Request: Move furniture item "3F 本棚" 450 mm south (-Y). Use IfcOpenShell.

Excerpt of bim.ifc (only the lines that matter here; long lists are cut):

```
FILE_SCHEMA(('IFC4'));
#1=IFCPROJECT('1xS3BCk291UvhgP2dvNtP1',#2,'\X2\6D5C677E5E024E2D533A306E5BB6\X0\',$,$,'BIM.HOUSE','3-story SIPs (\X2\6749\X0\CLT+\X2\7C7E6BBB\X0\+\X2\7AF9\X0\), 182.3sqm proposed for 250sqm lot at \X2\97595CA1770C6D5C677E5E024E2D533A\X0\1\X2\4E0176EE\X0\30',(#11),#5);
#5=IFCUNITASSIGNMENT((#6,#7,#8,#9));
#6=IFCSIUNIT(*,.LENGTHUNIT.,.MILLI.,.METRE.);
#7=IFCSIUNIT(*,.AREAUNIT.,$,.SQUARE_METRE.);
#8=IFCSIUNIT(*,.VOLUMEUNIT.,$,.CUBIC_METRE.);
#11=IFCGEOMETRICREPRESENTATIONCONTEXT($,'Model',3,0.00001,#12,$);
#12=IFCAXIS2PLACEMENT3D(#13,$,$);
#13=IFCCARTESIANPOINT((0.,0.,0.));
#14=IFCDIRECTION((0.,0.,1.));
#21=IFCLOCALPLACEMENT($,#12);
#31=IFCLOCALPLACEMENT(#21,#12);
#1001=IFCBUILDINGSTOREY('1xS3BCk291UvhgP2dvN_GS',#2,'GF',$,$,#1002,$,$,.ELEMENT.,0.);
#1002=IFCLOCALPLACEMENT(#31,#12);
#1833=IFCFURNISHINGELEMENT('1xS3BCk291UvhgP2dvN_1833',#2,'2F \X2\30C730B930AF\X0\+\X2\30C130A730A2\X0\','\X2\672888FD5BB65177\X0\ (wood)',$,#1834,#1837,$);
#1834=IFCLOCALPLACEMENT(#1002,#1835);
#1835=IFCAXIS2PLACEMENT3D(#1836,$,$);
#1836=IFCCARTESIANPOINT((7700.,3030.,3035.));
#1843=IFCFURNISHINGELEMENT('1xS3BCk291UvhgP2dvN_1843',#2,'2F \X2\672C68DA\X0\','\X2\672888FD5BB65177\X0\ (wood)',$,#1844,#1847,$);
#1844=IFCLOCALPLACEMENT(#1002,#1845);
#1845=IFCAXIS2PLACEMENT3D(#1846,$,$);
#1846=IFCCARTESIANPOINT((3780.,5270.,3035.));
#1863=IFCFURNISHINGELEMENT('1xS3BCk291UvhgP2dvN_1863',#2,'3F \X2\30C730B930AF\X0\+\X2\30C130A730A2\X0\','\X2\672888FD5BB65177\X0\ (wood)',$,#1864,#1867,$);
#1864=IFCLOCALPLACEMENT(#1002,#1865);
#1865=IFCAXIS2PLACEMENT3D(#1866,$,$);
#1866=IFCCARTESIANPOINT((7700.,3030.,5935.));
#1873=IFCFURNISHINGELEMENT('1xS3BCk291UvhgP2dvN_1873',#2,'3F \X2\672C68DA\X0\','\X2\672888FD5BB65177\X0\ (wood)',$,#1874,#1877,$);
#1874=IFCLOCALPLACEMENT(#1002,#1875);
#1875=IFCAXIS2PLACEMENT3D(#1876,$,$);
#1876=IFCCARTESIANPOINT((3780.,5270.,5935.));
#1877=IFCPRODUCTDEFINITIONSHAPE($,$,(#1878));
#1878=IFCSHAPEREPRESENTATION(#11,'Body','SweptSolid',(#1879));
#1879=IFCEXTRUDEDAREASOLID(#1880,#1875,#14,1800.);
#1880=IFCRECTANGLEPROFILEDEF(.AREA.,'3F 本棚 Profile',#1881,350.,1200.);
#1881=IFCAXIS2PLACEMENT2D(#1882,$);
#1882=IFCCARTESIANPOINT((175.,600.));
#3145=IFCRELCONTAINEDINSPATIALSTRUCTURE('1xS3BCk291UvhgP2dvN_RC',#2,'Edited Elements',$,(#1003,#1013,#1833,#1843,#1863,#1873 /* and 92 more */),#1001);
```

```python
import ifcopenshell
import ifcopenshell.api.geometry
import ifcopenshell.util.placement

model = ifcopenshell.open("bim.ifc")

item = model.by_id(1873)
matrix = ifcopenshell.util.placement.get_local_placement(item.ObjectPlacement)
matrix[1, 3] -= 450.0
ifcopenshell.api.geometry.edit_object_placement(model, product=item, matrix=matrix, is_si=False)

print(ifcopenshell.util.placement.get_local_placement(item.ObjectPlacement).round(3) + 0.0)

model.write("bim-out.ifc")
```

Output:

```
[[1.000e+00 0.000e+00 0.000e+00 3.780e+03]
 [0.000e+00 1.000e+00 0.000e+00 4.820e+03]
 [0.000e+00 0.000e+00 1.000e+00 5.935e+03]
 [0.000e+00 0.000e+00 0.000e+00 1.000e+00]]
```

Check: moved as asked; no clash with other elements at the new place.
